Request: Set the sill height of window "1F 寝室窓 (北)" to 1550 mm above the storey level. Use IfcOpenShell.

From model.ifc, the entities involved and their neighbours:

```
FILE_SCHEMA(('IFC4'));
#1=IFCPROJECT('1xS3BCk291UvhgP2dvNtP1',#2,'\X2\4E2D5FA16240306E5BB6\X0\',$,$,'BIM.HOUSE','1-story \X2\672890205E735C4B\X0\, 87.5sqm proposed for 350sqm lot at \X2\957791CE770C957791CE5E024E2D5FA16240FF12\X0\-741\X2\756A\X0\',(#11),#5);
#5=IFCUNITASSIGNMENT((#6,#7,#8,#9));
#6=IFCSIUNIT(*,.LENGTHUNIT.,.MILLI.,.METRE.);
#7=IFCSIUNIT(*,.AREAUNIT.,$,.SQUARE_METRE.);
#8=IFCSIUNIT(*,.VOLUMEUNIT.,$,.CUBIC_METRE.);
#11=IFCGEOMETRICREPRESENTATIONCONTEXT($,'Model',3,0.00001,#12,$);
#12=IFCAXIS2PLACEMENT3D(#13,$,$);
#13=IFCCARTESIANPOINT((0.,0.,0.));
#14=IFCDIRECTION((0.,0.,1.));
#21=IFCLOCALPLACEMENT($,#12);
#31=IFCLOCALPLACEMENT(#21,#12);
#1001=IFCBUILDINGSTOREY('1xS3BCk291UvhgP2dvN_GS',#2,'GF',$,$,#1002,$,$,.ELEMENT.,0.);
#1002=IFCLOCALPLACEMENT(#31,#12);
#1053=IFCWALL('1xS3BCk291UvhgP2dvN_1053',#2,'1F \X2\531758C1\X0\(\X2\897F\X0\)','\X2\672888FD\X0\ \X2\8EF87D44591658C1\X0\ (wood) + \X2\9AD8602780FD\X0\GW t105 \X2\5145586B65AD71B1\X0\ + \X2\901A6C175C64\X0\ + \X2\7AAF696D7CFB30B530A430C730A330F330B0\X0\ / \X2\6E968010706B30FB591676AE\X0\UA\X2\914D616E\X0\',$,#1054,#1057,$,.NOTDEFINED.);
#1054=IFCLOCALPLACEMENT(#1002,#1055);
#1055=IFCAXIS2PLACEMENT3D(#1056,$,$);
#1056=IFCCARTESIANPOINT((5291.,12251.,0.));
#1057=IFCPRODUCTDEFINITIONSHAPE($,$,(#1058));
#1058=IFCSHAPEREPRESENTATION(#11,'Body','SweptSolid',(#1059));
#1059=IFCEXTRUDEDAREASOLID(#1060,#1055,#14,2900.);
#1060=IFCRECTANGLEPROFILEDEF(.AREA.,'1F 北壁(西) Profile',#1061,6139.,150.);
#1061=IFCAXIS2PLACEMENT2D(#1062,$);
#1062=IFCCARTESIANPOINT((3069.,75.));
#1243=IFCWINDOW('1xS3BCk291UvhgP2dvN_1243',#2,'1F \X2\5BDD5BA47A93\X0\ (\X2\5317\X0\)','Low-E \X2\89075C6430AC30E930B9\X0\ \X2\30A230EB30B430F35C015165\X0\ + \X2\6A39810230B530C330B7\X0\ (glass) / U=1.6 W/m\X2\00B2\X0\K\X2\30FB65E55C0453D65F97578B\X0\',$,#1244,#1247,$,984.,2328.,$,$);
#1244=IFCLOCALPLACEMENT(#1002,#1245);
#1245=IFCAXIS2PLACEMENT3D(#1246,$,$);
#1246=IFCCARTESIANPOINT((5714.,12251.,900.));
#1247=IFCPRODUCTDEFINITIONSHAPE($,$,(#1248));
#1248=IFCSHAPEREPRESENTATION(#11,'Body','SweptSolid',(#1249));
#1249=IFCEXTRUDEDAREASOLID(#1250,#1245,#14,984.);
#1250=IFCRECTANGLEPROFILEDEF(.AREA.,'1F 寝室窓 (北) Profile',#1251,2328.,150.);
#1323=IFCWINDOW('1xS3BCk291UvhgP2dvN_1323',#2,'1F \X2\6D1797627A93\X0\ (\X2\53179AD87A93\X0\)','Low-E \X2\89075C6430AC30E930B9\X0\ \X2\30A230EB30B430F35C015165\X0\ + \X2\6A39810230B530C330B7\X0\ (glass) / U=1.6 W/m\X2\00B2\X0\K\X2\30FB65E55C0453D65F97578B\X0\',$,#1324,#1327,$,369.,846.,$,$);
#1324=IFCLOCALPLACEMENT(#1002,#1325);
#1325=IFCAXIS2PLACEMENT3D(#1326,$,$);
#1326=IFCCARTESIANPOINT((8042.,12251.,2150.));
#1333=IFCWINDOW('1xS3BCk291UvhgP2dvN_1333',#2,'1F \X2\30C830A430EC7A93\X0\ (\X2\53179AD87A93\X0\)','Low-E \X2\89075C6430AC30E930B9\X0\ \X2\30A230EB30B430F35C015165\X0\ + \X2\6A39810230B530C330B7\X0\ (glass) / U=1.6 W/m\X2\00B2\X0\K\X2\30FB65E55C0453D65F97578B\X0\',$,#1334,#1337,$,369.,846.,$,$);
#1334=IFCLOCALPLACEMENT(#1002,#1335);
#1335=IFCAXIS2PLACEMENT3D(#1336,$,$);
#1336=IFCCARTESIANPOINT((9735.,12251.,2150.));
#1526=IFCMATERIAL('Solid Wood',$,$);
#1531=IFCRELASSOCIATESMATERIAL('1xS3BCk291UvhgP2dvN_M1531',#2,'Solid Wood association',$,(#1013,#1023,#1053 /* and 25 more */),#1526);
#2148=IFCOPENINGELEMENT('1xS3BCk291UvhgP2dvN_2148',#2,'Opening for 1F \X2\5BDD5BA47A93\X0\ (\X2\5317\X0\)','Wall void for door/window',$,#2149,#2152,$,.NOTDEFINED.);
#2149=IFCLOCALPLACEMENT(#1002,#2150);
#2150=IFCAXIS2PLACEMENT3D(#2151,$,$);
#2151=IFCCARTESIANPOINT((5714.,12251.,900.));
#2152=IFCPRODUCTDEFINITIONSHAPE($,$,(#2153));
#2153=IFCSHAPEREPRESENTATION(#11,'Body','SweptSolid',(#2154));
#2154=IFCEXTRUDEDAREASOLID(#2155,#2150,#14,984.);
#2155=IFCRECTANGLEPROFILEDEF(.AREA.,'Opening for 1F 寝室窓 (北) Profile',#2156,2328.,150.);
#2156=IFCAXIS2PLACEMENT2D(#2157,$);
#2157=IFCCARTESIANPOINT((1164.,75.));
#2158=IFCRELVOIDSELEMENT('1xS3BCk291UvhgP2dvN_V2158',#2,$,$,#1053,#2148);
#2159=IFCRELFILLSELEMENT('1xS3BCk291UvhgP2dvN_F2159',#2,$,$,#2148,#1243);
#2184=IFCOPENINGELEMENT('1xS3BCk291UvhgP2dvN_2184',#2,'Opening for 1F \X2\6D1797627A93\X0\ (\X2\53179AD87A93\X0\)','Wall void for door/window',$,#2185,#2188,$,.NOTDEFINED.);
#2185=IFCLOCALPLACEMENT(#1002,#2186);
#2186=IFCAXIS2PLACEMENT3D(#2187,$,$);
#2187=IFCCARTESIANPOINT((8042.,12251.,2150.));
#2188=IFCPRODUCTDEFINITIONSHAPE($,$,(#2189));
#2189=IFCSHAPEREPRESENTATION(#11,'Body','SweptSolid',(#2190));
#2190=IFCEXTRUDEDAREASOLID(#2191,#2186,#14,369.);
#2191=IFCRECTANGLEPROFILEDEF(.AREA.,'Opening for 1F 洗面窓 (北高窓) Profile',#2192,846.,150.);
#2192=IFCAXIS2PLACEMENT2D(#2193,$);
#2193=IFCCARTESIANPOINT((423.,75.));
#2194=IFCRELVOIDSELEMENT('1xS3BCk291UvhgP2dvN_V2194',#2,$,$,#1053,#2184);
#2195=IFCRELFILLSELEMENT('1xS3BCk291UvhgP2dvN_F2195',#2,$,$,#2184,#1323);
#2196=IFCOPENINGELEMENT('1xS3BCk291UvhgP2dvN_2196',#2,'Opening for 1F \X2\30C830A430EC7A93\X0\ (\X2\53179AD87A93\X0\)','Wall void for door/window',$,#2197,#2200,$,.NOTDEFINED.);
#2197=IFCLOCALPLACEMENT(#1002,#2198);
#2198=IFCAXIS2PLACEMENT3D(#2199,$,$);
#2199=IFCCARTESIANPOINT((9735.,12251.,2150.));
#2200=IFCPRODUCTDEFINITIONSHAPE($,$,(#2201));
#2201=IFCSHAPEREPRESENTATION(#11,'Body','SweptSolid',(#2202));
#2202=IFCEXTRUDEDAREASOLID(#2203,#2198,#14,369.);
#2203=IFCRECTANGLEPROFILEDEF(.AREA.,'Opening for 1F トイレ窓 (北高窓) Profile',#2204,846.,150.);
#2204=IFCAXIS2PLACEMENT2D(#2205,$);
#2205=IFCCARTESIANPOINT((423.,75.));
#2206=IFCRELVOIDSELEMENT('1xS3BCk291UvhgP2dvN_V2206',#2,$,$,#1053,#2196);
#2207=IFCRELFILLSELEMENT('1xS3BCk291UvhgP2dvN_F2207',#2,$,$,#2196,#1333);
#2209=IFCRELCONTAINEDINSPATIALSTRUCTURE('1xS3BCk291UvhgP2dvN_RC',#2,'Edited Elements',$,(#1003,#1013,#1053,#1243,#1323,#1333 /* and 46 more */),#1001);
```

```python
import numpy as np
import ifcopenshell
import ifcopenshell.api.geometry
import ifcopenshell.geom
import ifcopenshell.util.element
import ifcopenshell.util.placement
import ifcopenshell.util.shape
import ifcopenshell.util.unit

model = ifcopenshell.open("model.ifc")
unit_scale = ifcopenshell.util.unit.calculate_unit_scale(model)

window = model.by_guid("1xS3BCk291UvhgP2dvN_1243")
opening = window.FillsVoids[0].RelatingOpeningElement
storey = ifcopenshell.util.element.get_container(window, ifc_class="IfcBuildingStorey")
level = ifcopenshell.util.placement.get_local_placement(storey.ObjectPlacement)[2, 3]

# The opening's origin need not be at the sill, so measure its lowest point.
shape = ifcopenshell.geom.create_shape(ifcopenshell.geom.settings(), opening)
bottom = ifcopenshell.util.shape.get_shape_bottom_elevation(shape, shape.geometry) / unit_scale
dz = level + 1.55 / unit_scale - bottom

shift = np.array([0.0, 0.0, dz])
# The window is not placed relative to its opening, so move both.
for product in (opening, window):
    matrix = ifcopenshell.util.placement.get_local_placement(product.ObjectPlacement)
    matrix[:3, 3] += shift
    ifcopenshell.api.geometry.edit_object_placement(model, product=product, matrix=matrix, is_si=False)

print(f"moved by {dz * unit_scale:+.3f} m")

model.write("model_v2.ifc")
```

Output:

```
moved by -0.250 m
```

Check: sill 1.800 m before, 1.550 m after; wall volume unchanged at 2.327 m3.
